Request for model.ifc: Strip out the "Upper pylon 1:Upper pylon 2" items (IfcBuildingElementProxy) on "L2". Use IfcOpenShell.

First a look at what the model holds.

```python
import ifcopenshell
import ifcopenshell.util.element

model = ifcopenshell.open("model.ifc")
print(model.schema)
storey = next(s for s in model.by_type("IfcBuildingStorey") if s.Name == "L2")
proxies = [e for e in ifcopenshell.util.element.get_decomposition(storey) if e.is_a("IfcBuildingElementProxy")]
seen = {}
for e in proxies:
    element_type = ifcopenshell.util.element.get_type(e)
    name = element_type.Name if element_type not in (None, e) else None
    seen[name] = seen.get(name, 0) + 1
for name, count in sorted(seen.items(), key=str):
    print(count, "x", name)
```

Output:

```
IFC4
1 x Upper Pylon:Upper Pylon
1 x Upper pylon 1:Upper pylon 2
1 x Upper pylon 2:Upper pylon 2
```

```python
import ifcopenshell
import ifcopenshell.api.root
import ifcopenshell.util.element

model = ifcopenshell.open("model.ifc")

storey = next(s for s in model.by_type("IfcBuildingStorey") if s.Name == "L2")
proxies = [e for e in ifcopenshell.util.element.get_decomposition(storey) if e.is_a("IfcBuildingElementProxy")]
targets = [e for e in proxies if (t := ifcopenshell.util.element.get_type(e)) not in (None, e) and t.Name == "Upper pylon 1:Upper pylon 2"]

for e in targets:
    ifcopenshell.api.root.remove_product(model, product=e)
print(len(targets), "removed")

model.write("model_rev.ifc")
```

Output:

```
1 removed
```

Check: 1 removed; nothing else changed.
